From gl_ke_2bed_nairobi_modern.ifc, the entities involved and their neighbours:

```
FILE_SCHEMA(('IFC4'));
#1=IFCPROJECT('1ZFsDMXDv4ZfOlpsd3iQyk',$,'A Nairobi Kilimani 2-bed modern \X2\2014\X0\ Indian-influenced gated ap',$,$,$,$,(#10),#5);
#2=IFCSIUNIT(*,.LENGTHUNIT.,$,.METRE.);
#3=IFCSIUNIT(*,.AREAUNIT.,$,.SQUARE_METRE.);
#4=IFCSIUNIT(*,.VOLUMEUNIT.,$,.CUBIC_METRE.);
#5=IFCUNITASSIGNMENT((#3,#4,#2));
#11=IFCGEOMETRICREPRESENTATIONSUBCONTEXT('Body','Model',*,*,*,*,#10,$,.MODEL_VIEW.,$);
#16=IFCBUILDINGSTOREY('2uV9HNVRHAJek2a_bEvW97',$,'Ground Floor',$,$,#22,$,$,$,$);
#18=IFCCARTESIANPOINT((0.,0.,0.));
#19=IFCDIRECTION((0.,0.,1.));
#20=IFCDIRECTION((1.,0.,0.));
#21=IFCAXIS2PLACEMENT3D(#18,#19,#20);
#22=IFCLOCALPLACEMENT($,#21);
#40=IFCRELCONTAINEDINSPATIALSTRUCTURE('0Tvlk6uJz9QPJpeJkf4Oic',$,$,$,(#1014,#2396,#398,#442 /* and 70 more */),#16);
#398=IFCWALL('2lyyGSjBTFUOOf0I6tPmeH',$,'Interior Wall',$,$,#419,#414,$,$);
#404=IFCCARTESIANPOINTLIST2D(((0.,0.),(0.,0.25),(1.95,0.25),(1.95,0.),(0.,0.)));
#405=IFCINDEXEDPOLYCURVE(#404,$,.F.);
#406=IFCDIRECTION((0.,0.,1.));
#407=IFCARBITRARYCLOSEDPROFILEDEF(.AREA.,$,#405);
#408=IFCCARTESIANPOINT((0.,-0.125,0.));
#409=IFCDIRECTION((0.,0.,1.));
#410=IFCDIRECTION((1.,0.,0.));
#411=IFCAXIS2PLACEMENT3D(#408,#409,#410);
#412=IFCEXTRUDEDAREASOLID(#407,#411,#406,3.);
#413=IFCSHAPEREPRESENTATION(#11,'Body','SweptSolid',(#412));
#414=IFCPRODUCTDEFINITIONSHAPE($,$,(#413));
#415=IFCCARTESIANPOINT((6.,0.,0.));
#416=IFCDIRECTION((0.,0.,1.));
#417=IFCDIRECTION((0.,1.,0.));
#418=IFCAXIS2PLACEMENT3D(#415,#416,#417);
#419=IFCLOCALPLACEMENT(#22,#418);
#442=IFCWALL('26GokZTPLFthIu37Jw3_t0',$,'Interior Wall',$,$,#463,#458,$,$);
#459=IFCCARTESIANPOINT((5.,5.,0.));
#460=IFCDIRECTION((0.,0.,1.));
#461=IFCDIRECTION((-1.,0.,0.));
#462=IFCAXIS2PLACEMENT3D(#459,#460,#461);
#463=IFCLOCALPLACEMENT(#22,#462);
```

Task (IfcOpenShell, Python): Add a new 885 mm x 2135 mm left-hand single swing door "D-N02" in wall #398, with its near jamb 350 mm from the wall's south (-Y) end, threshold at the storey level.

```python
import numpy as np
import ifcopenshell
import ifcopenshell.api.feature
import ifcopenshell.api.geometry
import ifcopenshell.api.root
import ifcopenshell.api.spatial
import ifcopenshell.geom
import ifcopenshell.util.element
import ifcopenshell.util.placement
import ifcopenshell.util.representation
import ifcopenshell.util.shape
import ifcopenshell.util.unit

model = ifcopenshell.open("gl_ke_2bed_nairobi_modern.ifc")
unit_scale = ifcopenshell.util.unit.calculate_unit_scale(model)
settings = ifcopenshell.geom.settings()


def volume(element):
    """Net volume in cubic metres, openings subtracted."""
    shape = ifcopenshell.geom.create_shape(settings, element)
    return ifcopenshell.util.shape.get_volume(shape.geometry)


wall = model.by_guid("2lyyGSjBTFUOOf0I6tPmeH")
storey = ifcopenshell.util.element.get_container(wall, ifc_class="IfcBuildingStorey")
context = ifcopenshell.util.representation.get_context(model, "Model", "Body", "MODEL_VIEW")
before = volume(wall)

width, height, from_end, sill = 0.885, 2.135, 0.35, 0.0  # metres

# The wall runs along its own X axis, and the end named is its -X end.
wall_shape = ifcopenshell.geom.create_shape(settings, wall)
x, y, z = ifcopenshell.util.shape.get_vertices(wall_shape.geometry).T
start = x.min() + from_end
face, thickness = float(y.min()), float(y.max() - y.min())
wall_matrix = ifcopenshell.util.placement.get_local_placement(wall.ObjectPlacement)
level = ifcopenshell.util.placement.get_local_placement(storey.ObjectPlacement)[2, 3]


def in_wall(x, y):
    """Placement at x, y metres in the wall's axes, at sill height."""
    matrix = wall_matrix.copy()
    matrix[:, 3] = wall_matrix @ np.array([x / unit_scale, y / unit_scale, 0.0, 1.0])
    matrix[2, 3] = level + sill / unit_scale
    return matrix


# Opening: a box that overshoots both wall faces by 50 mm.
opening = ifcopenshell.api.root.create_entity(model, ifc_class="IfcOpeningElement", predefined_type="OPENING")
box = ifcopenshell.api.geometry.add_wall_representation(
    model, context=context, length=width, height=height, thickness=thickness + 0.1
)
ifcopenshell.api.geometry.assign_representation(model, product=opening, representation=box)
ifcopenshell.api.geometry.edit_object_placement(model, product=opening, matrix=in_wall(start, face - 0.05), is_si=False)
ifcopenshell.api.feature.add_feature(model, feature=opening, element=wall)

door = ifcopenshell.api.root.create_entity(model, ifc_class="IfcDoor", name="D-N02", predefined_type="DOOR")
door.OverallWidth, door.OverallHeight = width / unit_scale, height / unit_scale
door.OperationType = "SINGLE_SWING_LEFT"
body = ifcopenshell.api.geometry.add_door_representation(
    model,
    context=context,
    overall_width=door.OverallWidth,
    overall_height=door.OverallHeight,
    operation_type="SINGLE_SWING_LEFT",
    lining_properties={"LiningDepth": thickness / unit_scale, "ThresholdDepth": thickness / unit_scale},
)
ifcopenshell.api.geometry.assign_representation(model, product=door, representation=body)
ifcopenshell.api.spatial.assign_container(model, products=[door], relating_structure=storey)
ifcopenshell.api.feature.add_filling(model, opening=opening, element=door)

# The lining spans the wall, so the door starts at the wall face.
ifcopenshell.api.geometry.edit_object_placement(model, product=door, matrix=in_wall(start, face), is_si=False)

after = volume(wall)

print(f"wall volume {before:.3f} -> {after:.3f} m3")

model.write("gl_ke_2bed_nairobi_modern_edited.ifc")
```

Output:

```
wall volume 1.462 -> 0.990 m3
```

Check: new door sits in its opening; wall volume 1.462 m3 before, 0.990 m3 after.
